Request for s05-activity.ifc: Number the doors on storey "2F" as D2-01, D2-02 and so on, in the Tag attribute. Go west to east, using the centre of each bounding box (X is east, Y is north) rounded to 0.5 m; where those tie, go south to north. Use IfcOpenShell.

First a look at what the model holds.

```python
import ifcopenshell
import ifcopenshell.util.element
import ifcopenshell.util.placement

model = ifcopenshell.open("s05-activity.ifc")
print(model.schema)
storey = next(s for s in model.by_type("IfcBuildingStorey") if s.Name == "2F")
doors = [e for e in ifcopenshell.util.element.get_decomposition(storey) if e.is_a("IfcDoor")]
for e in sorted(doors, key=lambda e: e.id()):
    origin = ifcopenshell.util.placement.get_local_placement(e.ObjectPlacement)[:3, 3]
    print(e.id(), e.Tag, e.Name, origin.round(2) + 0.0, sep=" | ")
```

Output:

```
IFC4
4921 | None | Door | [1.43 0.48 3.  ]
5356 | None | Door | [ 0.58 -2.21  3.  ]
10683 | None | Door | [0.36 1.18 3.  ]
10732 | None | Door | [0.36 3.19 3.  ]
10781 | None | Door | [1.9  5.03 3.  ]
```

```python
import ifcopenshell
import ifcopenshell.geom
import ifcopenshell.util.element
import ifcopenshell.util.shape

model = ifcopenshell.open("s05-activity.ifc")
settings = ifcopenshell.geom.settings()
settings.set("use-world-coords", True)


def centre(element):
    shape = ifcopenshell.geom.create_shape(settings, element)
    return ifcopenshell.util.shape.get_bbox_centroid(shape.geometry)


storey = next(s for s in model.by_type("IfcBuildingStorey") if s.Name == "2F")
doors = [e for e in ifcopenshell.util.element.get_decomposition(storey) if e.is_a("IfcDoor")]

# Insertion points can sit at a corner or the storey origin, so sort by the geometry (in metres).
centres = {e: centre(e) for e in doors}
doors.sort(key=lambda e: (round(centres[e][0] / 0.5), centres[e][1]))

for i, e in enumerate(doors, start=1):
    number = f"D2-{i:02d}"
    e.Tag = number
    print(e.id(), number)

model.write("s05-activity_v2.ifc")
```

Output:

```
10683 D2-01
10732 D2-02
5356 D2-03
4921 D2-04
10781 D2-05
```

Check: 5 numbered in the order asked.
